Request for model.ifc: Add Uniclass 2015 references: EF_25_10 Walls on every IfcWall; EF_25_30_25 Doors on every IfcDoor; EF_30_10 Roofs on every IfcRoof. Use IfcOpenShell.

First a look at what the model holds.

```python
import ifcopenshell

model = ifcopenshell.open("model.ifc")
print(model.schema)
print("classifications:", [c.Name for c in model.by_type("IfcClassification")])
for ifc_class in ("IfcDoor", "IfcRoof", "IfcStair", "IfcWall", "IfcWindow"):
    print(ifc_class, len(model.by_type(ifc_class)))
```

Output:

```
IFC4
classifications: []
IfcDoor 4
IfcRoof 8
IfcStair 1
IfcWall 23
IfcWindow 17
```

```python
import ifcopenshell
import ifcopenshell.api.classification

model = ifcopenshell.open("model.ifc")

system = ifcopenshell.api.classification.add_classification(model, classification="Uniclass 2015")

codes = {
    "IfcWall": ("EF_25_10", "Walls"),
    "IfcDoor": ("EF_25_30_25", "Doors"),
    "IfcRoof": ("EF_30_10", "Roofs"),
}
for ifc_class, (code, name) in codes.items():
    products = model.by_type(ifc_class)
    ifcopenshell.api.classification.add_reference(
        model, products=products, classification=system, identification=code, name=name
    )
    print(code, len(products))

model.write("model-out.ifc")
```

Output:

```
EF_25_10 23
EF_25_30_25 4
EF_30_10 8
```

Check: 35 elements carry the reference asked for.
